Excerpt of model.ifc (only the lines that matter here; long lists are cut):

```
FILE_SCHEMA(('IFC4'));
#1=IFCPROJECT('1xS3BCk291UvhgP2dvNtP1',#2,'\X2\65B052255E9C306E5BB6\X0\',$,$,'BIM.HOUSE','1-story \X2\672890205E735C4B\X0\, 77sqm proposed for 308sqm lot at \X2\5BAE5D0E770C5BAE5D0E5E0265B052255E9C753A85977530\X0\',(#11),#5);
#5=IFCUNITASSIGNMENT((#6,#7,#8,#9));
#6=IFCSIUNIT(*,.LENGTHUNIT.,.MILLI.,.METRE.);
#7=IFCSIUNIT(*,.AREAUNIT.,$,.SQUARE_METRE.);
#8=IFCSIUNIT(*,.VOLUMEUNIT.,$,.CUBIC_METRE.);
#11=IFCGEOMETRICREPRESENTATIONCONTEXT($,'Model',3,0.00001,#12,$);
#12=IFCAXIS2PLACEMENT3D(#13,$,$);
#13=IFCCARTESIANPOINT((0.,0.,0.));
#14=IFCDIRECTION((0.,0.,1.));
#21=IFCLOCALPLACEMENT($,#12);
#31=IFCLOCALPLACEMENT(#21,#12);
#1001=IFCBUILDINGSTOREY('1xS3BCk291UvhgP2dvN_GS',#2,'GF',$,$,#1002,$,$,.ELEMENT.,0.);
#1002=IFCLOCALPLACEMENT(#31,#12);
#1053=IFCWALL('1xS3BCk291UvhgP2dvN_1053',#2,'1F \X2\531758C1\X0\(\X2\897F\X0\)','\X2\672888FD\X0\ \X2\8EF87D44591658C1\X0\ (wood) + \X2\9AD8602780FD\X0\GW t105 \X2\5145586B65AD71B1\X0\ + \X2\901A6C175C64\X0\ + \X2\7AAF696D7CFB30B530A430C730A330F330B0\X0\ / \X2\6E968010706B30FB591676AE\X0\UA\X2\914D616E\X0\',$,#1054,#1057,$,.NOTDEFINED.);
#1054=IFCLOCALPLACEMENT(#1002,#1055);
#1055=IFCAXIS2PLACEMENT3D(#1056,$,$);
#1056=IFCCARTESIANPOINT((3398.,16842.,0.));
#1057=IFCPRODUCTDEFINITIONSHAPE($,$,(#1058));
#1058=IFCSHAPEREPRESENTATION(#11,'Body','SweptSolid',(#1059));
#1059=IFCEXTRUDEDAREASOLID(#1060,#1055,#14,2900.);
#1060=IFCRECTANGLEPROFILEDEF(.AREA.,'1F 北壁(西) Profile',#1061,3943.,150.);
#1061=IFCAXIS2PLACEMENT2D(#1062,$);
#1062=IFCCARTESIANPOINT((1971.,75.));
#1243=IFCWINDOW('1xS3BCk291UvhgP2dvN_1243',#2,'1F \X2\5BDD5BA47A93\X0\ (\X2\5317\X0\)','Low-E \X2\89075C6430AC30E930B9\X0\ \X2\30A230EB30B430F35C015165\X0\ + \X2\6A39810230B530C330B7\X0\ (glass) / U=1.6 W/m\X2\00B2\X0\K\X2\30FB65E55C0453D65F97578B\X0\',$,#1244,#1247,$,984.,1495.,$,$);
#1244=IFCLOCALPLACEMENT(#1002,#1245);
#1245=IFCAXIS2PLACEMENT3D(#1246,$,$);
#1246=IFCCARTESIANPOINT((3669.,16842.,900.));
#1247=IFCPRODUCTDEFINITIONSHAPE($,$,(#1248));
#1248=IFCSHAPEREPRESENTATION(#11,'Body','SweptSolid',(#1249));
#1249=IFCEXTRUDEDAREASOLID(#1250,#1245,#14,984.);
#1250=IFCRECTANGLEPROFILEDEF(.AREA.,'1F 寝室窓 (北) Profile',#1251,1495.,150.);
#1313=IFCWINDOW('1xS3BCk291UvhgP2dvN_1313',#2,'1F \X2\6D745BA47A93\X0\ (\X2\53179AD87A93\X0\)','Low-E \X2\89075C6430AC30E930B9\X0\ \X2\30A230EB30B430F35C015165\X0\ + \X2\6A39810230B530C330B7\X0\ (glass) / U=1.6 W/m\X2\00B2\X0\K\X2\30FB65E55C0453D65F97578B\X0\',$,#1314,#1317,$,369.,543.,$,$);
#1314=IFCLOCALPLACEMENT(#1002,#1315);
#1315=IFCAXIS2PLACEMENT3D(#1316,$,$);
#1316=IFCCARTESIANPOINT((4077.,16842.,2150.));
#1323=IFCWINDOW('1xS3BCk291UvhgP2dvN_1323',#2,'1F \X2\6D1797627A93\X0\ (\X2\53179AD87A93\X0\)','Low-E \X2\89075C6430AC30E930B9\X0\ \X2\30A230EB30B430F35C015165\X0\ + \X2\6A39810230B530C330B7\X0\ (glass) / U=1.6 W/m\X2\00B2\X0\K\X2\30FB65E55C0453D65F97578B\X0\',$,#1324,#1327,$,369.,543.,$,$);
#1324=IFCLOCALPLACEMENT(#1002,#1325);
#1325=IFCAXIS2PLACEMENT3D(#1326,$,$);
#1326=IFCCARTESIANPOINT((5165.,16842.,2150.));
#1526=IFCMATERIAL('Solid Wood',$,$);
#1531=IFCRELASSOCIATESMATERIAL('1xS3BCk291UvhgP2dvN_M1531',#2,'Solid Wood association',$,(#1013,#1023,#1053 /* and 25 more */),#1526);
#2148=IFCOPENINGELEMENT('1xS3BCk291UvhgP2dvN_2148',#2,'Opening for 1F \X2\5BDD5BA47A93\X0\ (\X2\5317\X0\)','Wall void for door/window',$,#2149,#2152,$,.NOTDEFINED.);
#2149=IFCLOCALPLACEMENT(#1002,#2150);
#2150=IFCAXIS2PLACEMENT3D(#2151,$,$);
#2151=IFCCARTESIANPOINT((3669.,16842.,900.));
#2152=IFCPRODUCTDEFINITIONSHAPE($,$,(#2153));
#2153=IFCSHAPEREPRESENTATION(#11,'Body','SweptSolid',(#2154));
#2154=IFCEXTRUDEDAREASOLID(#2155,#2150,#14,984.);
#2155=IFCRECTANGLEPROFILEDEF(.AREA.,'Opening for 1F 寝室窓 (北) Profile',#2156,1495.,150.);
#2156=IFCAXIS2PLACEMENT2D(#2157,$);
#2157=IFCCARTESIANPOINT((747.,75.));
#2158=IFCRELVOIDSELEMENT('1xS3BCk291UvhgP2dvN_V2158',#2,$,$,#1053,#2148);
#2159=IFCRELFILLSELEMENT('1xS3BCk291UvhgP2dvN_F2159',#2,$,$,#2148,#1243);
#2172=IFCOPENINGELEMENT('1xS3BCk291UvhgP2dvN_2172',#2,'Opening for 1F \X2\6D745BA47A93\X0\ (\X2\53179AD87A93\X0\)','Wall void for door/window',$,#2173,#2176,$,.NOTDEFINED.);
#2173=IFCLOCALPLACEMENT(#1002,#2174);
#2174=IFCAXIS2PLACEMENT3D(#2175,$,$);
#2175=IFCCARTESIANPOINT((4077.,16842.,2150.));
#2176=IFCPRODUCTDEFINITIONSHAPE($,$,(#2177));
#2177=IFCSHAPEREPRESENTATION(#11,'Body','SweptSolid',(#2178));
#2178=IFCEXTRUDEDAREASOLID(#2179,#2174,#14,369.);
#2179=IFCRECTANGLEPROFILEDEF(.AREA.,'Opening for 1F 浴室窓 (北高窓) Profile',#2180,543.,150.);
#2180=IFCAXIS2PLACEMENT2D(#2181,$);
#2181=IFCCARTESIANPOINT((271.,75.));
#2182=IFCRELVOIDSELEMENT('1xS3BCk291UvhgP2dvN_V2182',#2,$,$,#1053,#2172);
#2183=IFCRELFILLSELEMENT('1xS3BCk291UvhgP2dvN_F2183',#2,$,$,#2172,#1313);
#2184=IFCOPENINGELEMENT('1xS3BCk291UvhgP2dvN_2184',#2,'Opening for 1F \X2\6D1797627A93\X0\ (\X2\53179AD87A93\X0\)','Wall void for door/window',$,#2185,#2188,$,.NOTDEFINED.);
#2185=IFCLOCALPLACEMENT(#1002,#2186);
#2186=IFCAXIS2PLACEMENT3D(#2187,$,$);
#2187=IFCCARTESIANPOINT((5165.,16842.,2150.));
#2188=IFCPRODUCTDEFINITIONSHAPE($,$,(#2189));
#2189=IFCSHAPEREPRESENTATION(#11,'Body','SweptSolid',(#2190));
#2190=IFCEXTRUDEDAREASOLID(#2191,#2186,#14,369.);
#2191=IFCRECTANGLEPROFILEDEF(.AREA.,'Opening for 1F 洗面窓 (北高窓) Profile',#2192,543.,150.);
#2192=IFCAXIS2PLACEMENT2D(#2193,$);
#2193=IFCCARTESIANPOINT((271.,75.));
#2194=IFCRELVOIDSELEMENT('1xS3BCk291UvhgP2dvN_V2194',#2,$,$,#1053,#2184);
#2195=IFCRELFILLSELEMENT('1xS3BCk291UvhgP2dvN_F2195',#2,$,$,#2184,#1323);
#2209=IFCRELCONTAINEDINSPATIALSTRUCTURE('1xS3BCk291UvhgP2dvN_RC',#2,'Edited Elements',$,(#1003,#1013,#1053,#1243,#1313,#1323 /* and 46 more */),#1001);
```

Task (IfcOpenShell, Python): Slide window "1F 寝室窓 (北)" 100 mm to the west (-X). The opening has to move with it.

```python
import ifcopenshell
import ifcopenshell.api.geometry
import ifcopenshell.util.placement

model = ifcopenshell.open("model.ifc")

window = model.by_guid("1xS3BCk291UvhgP2dvN_1243")
opening = window.FillsVoids[0].RelatingOpeningElement
wall = opening.VoidsElements[0].RelatingBuildingElement

wall_matrix = ifcopenshell.util.placement.get_local_placement(wall.ObjectPlacement)
shift = wall_matrix[:3, 0] * -100.0
before = ifcopenshell.util.placement.get_local_placement(window.ObjectPlacement)[:3, 3].copy()

# The window is not placed relative to its opening, so move both.
for product in (opening, window):
    matrix = ifcopenshell.util.placement.get_local_placement(product.ObjectPlacement)
    matrix[:3, 3] += shift
    ifcopenshell.api.geometry.edit_object_placement(model, product=product, matrix=matrix, is_si=False)

after = ifcopenshell.util.placement.get_local_placement(window.ObjectPlacement)[:3, 3]
print("window moved by", (after - before).round(3) + 0.0)

model.write("model-out.ifc")
```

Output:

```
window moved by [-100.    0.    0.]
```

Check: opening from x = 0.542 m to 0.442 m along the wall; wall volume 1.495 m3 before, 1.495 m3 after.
